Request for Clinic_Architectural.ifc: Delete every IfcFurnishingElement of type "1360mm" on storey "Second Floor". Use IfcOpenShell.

First a look at what the model holds.

```python
import ifcopenshell
import ifcopenshell.util.element

model = ifcopenshell.open("Clinic_Architectural.ifc")
print(model.schema)
storey = next(s for s in model.by_type("IfcBuildingStorey") if s.Name == "Second Floor")
furniture = [e for e in ifcopenshell.util.element.get_decomposition(storey) if e.is_a("IfcFurnishingElement")]
seen = {}
for e in furniture:
    element_type = ifcopenshell.util.element.get_type(e)
    name = element_type.Name if element_type not in (None, e) else None
    seen[name] = seen.get(name, 0) + 1
for name, count in sorted(seen.items(), key=str):
    print(count, "x", name)
```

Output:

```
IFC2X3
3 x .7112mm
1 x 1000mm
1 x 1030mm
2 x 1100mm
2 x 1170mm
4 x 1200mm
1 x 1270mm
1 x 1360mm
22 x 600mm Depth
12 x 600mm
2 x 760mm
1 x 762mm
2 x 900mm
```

```python
import ifcopenshell
import ifcopenshell.api.root
import ifcopenshell.util.element

model = ifcopenshell.open("Clinic_Architectural.ifc")

storey = next(s for s in model.by_type("IfcBuildingStorey") if s.Name == "Second Floor")
furniture = [e for e in ifcopenshell.util.element.get_decomposition(storey) if e.is_a("IfcFurnishingElement")]
targets = [e for e in furniture if (t := ifcopenshell.util.element.get_type(e)) not in (None, e) and t.Name == "1360mm"]

for e in targets:
    ifcopenshell.api.root.remove_product(model, product=e)
print(len(targets), "removed")

model.write("Clinic_Architectural_updated.ifc")
```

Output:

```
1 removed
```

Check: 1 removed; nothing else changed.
